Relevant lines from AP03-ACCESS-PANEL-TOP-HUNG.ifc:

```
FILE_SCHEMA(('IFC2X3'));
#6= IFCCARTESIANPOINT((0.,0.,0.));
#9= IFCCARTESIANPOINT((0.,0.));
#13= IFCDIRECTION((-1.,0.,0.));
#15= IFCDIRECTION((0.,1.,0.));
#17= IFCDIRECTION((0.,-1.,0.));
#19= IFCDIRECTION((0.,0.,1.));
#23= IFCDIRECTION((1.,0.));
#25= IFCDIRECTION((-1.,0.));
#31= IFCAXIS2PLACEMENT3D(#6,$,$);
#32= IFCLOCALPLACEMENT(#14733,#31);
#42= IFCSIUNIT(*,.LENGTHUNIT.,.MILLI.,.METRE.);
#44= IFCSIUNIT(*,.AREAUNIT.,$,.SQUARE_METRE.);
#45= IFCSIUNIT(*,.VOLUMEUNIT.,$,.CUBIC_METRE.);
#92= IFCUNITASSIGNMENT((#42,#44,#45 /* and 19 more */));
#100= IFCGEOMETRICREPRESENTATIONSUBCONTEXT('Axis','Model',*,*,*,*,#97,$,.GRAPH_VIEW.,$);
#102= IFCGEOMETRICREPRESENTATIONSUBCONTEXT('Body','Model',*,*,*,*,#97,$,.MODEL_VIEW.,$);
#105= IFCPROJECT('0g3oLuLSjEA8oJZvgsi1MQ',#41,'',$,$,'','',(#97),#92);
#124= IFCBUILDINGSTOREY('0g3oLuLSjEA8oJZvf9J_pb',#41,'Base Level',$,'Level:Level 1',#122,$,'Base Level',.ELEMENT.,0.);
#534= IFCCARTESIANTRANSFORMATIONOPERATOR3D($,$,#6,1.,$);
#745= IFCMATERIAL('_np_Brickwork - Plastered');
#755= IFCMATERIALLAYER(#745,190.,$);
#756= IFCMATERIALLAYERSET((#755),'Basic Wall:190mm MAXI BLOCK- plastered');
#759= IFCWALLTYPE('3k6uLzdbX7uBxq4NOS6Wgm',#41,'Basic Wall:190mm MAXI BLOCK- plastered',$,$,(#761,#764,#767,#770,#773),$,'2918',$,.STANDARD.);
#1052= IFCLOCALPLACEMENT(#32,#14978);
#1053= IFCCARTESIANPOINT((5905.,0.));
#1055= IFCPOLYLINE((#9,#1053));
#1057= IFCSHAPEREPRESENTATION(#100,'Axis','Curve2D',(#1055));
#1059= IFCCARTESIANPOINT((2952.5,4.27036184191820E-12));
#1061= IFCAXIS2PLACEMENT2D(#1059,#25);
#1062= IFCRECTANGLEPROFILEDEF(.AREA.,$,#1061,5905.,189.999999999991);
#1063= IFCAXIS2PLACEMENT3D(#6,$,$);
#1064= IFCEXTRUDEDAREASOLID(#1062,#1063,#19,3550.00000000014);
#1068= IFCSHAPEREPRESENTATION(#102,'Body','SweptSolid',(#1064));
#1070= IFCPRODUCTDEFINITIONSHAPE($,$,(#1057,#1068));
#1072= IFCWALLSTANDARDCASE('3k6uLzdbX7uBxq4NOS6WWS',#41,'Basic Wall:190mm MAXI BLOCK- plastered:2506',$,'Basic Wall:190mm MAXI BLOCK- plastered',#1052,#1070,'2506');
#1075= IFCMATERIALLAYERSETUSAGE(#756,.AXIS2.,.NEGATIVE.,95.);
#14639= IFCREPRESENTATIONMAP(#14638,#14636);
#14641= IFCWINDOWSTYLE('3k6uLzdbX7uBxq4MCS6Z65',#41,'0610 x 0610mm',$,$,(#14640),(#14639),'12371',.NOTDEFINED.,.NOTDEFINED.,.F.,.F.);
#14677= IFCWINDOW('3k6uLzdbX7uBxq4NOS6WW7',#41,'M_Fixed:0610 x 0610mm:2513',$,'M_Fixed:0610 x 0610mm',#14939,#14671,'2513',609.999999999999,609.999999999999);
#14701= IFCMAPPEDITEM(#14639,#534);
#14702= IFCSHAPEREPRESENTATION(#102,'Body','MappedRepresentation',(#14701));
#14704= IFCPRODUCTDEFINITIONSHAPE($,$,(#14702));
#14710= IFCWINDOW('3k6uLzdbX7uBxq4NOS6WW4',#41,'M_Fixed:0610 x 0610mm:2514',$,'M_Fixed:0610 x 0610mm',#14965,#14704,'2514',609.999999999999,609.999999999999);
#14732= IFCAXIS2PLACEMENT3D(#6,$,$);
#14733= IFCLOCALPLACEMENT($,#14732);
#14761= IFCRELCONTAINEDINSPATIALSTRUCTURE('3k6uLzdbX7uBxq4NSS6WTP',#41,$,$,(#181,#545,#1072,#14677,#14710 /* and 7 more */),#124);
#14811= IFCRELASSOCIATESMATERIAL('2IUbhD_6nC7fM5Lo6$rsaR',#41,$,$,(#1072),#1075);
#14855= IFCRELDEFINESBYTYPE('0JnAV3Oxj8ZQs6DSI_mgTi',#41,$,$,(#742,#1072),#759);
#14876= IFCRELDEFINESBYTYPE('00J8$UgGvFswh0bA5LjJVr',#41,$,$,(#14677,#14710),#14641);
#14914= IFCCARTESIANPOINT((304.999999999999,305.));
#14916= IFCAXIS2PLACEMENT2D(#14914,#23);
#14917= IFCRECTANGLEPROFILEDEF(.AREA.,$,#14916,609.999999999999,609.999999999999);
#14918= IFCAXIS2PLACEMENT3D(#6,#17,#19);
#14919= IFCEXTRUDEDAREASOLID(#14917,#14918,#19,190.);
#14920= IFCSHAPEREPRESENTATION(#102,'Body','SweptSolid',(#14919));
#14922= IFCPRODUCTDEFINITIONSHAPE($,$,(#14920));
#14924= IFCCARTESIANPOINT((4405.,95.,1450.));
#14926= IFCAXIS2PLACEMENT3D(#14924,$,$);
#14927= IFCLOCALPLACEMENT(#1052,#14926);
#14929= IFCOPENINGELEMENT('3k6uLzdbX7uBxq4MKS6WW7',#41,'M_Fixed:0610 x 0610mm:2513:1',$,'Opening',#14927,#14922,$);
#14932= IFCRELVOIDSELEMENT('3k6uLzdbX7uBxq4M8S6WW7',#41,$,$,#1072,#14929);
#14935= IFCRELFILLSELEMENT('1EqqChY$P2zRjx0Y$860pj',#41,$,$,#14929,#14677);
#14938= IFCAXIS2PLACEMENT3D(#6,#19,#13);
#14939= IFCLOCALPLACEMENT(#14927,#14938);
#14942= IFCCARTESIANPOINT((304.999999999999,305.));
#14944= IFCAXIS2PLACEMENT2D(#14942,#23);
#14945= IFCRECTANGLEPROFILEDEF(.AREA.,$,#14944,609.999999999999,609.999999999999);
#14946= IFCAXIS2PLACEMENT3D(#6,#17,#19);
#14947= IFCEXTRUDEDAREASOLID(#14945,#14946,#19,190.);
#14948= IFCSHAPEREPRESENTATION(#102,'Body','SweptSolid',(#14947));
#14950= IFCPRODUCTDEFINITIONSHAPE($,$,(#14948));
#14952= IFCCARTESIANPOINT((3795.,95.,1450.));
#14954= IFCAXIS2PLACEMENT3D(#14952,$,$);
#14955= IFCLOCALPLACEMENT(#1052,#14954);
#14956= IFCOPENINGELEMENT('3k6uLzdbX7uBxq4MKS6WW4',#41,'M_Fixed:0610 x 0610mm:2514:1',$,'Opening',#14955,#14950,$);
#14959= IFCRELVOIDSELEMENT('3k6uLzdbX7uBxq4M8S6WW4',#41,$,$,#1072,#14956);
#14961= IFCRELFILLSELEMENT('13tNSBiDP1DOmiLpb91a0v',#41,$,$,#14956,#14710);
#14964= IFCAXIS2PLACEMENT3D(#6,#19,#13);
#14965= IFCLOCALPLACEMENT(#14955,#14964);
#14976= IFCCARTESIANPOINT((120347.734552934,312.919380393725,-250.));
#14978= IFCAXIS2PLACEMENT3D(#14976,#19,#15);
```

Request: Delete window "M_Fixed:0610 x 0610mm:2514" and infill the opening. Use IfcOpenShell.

```python
import ifcopenshell
import ifcopenshell.api.feature
import ifcopenshell.api.root
import ifcopenshell.geom
import ifcopenshell.util.shape

model = ifcopenshell.open("AP03-ACCESS-PANEL-TOP-HUNG.ifc")
settings = ifcopenshell.geom.settings()


def volume(element):
    """Net volume in cubic metres, openings subtracted."""
    shape = ifcopenshell.geom.create_shape(settings, element)
    return ifcopenshell.util.shape.get_volume(shape.geometry)


window = model.by_guid("3k6uLzdbX7uBxq4NOS6WW4")
opening = window.FillsVoids[0].RelatingOpeningElement
wall = opening.VoidsElements[0].RelatingBuildingElement
before = volume(wall)

ifcopenshell.api.root.remove_product(model, product=window)
ifcopenshell.api.feature.remove_feature(model, feature=opening)

after = volume(wall)

print(f"wall volume {before:.3f} -> {after:.3f} m3")

model.write("AP03-ACCESS-PANEL-TOP-HUNG_rev.ifc")
```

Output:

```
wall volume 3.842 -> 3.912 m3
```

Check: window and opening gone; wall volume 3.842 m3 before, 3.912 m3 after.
